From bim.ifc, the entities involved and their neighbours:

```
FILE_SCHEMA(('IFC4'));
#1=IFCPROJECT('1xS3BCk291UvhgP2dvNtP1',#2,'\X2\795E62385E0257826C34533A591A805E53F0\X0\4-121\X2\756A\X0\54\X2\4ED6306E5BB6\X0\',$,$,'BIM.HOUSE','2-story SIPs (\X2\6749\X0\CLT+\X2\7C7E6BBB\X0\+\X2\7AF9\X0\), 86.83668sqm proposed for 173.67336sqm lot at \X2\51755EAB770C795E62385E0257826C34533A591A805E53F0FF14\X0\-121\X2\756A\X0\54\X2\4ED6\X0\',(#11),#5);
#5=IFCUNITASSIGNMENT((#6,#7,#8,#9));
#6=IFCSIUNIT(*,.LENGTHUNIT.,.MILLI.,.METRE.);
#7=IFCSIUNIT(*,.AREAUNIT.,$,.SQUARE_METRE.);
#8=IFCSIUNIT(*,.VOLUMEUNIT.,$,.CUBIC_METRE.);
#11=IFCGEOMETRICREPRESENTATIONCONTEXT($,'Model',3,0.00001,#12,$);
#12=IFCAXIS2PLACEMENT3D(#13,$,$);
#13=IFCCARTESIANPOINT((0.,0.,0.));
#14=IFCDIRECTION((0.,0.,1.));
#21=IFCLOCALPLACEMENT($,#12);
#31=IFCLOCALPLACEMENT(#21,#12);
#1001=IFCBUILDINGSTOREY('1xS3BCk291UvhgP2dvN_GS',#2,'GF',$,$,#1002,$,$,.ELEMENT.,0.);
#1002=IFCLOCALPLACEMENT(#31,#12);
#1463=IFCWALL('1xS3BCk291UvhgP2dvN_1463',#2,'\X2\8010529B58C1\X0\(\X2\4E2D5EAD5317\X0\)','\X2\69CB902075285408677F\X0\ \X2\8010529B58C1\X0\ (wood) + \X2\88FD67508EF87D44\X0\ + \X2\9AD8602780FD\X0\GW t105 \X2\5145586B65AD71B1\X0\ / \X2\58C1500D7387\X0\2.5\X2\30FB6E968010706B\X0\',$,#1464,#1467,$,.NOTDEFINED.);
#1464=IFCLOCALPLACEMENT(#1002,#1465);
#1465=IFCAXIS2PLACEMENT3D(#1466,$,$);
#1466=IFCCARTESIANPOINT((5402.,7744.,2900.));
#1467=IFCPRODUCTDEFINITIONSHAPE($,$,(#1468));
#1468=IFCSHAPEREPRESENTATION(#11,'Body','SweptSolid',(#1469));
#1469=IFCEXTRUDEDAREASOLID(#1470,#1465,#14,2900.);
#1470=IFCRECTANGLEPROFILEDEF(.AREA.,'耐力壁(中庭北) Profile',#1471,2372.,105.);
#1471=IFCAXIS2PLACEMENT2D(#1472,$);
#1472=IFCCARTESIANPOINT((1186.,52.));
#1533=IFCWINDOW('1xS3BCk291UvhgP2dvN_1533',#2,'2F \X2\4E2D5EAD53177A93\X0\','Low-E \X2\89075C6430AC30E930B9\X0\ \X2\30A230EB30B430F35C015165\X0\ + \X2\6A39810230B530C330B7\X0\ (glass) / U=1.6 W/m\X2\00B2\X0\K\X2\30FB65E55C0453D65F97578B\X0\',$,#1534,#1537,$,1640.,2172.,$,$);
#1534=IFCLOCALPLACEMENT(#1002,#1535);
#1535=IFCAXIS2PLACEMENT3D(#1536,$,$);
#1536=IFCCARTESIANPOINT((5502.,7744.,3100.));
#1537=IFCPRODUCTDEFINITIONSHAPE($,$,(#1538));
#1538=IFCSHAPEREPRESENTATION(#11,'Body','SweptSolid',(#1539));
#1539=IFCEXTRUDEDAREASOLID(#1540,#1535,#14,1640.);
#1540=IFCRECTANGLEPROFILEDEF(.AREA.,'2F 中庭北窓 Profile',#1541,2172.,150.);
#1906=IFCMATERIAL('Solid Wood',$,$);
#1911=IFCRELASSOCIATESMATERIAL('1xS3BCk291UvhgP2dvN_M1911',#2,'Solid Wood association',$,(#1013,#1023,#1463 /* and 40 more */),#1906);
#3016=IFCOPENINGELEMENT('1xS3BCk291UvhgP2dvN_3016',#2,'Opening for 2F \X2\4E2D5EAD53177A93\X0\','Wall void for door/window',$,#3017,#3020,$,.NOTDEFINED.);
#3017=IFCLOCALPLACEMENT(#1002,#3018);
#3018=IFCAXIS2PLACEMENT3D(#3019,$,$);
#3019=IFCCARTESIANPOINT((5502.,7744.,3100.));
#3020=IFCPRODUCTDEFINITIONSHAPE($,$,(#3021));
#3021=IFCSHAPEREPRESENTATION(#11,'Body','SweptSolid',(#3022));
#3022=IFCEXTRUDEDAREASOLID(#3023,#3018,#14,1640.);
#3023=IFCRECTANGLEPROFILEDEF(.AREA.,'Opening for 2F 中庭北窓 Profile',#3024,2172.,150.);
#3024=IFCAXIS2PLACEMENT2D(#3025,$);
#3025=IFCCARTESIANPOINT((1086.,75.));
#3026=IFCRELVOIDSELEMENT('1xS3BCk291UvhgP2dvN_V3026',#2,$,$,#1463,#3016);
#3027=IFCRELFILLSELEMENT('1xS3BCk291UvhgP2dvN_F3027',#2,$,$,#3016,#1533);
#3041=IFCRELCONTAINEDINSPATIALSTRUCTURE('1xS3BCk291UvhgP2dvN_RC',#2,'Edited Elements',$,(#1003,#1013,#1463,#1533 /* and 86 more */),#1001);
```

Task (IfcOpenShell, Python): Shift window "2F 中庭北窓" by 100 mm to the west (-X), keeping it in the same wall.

```python
import ifcopenshell
import ifcopenshell.api.geometry
import ifcopenshell.util.placement

model = ifcopenshell.open("bim.ifc")

window = model.by_guid("1xS3BCk291UvhgP2dvN_1533")
opening = window.FillsVoids[0].RelatingOpeningElement
wall = opening.VoidsElements[0].RelatingBuildingElement

wall_matrix = ifcopenshell.util.placement.get_local_placement(wall.ObjectPlacement)
shift = wall_matrix[:3, 0] * -100.0
before = ifcopenshell.util.placement.get_local_placement(window.ObjectPlacement)[:3, 3].copy()

# The window is not placed relative to its opening, so move both.
for product in (opening, window):
    matrix = ifcopenshell.util.placement.get_local_placement(product.ObjectPlacement)
    matrix[:3, 3] += shift
    ifcopenshell.api.geometry.edit_object_placement(model, product=product, matrix=matrix, is_si=False)

after = ifcopenshell.util.placement.get_local_placement(window.ObjectPlacement)[:3, 3]
print("window moved by", (after - before).round(3) + 0.0)

model.write("bim_updated.ifc")
```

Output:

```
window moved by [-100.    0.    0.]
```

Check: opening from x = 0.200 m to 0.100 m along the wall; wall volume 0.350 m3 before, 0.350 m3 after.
